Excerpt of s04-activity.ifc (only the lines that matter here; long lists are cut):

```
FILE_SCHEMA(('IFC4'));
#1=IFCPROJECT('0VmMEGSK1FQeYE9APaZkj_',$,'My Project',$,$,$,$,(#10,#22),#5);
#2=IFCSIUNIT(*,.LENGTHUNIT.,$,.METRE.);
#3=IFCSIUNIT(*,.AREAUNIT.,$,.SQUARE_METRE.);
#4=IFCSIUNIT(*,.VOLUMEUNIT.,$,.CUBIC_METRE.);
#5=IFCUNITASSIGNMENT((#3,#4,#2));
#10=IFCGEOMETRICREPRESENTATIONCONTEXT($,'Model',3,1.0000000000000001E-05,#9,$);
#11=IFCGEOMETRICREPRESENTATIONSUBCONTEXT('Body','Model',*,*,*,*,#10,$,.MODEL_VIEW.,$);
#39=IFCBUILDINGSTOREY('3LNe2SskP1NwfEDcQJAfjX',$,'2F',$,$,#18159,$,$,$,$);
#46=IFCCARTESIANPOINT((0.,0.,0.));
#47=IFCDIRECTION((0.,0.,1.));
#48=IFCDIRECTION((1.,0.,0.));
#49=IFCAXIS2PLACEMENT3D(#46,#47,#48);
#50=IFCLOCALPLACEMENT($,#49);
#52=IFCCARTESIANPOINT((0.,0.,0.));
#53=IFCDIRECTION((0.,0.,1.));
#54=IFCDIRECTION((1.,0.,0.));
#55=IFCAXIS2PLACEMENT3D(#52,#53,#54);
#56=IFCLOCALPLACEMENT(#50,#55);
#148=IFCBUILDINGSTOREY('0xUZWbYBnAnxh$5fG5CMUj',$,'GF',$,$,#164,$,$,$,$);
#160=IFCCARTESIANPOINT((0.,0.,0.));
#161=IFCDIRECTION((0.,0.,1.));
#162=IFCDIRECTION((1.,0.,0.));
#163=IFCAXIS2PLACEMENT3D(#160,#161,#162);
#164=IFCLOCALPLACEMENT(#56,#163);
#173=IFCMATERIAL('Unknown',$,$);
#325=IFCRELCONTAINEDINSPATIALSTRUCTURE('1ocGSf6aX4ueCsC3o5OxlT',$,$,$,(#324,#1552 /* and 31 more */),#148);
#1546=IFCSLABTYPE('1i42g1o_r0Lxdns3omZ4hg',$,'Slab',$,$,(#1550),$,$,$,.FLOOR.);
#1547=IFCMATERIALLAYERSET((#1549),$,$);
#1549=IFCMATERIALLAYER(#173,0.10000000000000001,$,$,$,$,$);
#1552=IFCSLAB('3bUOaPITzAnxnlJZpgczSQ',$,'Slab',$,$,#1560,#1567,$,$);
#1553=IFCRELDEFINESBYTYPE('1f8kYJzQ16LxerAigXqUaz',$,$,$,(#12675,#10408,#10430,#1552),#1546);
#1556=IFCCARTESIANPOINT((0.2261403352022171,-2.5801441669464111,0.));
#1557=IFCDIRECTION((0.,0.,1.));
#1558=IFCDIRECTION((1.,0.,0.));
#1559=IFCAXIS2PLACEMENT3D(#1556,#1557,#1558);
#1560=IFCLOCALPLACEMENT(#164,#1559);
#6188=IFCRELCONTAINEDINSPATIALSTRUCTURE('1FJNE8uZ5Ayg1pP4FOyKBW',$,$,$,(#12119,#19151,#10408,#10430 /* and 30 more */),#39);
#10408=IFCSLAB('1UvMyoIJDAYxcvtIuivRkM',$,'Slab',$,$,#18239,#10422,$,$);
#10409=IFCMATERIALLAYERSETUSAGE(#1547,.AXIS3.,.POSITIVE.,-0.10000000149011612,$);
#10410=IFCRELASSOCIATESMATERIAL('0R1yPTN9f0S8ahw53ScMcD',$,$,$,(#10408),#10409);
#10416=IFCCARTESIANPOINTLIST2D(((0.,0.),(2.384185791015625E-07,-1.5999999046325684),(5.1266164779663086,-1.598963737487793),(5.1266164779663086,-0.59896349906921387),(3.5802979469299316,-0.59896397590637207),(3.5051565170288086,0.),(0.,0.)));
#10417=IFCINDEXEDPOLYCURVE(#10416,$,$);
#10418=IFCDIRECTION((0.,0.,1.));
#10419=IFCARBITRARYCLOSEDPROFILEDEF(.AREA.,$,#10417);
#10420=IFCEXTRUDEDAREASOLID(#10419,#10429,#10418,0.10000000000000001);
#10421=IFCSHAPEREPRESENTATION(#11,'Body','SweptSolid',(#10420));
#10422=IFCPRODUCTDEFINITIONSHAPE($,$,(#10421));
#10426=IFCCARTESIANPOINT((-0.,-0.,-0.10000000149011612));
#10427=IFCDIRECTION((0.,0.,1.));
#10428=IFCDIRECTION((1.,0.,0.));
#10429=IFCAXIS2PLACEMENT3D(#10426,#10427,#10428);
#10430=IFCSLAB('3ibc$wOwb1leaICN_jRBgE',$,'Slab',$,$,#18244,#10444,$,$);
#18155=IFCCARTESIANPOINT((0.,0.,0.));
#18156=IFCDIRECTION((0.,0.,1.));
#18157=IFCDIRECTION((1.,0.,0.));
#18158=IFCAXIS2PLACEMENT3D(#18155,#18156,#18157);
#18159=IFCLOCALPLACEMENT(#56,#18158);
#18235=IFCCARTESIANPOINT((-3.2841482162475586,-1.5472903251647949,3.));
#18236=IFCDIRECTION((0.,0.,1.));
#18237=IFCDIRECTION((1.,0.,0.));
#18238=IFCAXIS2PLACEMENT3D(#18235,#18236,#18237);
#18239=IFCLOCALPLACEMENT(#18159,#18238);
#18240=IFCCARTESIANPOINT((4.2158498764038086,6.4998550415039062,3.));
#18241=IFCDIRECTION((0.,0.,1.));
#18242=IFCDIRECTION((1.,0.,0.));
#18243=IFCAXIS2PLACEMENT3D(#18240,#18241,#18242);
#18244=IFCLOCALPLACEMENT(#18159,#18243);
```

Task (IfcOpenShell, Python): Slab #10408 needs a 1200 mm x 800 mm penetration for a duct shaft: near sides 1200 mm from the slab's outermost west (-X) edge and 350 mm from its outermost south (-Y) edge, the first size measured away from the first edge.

```python
import numpy as np
import ifcopenshell
import ifcopenshell.api.feature
import ifcopenshell.api.geometry
import ifcopenshell.api.root
import ifcopenshell.geom
import ifcopenshell.util.placement
import ifcopenshell.util.representation
import ifcopenshell.util.shape
import ifcopenshell.util.unit

model = ifcopenshell.open("s04-activity.ifc")
unit_scale = ifcopenshell.util.unit.calculate_unit_scale(model)
settings = ifcopenshell.geom.settings()


def volume(element):
    """Net volume in cubic metres, openings subtracted."""
    shape = ifcopenshell.geom.create_shape(settings, element)
    return ifcopenshell.util.shape.get_volume(shape.geometry)


slab = model.by_guid("1UvMyoIJDAYxcvtIuivRkM")
before = volume(slab)

# Extent in the slab's own axes, in metres. The edges named are its -X and -Y sides.
slab_shape = ifcopenshell.geom.create_shape(settings, slab)
vertices = ifcopenshell.util.shape.get_vertices(slab_shape.geometry)
x_min, y_min, bottom = vertices.min(axis=0)
top = vertices[:, 2].max()

opening = ifcopenshell.api.root.create_entity(model, ifc_class="IfcOpeningElement", name="Duct shaft opening", predefined_type="OPENING")
context = ifcopenshell.util.representation.get_context(model, "Model", "Body", "MODEL_VIEW")
width, depth = 1.2, 0.8
outline = [(0.0, 0.0), (width, 0.0), (width, depth), (0.0, depth), (0.0, 0.0)]
# Overshoot both faces by 50 mm so the cut is clean.
shape = ifcopenshell.api.geometry.add_slab_representation(
    model, context=context, depth=top - bottom + 0.1, polyline=outline
)
ifcopenshell.api.geometry.assign_representation(model, product=opening, representation=shape)

matrix = ifcopenshell.util.placement.get_local_placement(slab.ObjectPlacement)
matrix[:, 3] = matrix @ np.append(np.array([x_min + 1.2, y_min + 0.35, bottom - 0.05]) / unit_scale, 1.0)
ifcopenshell.api.geometry.edit_object_placement(model, product=opening, matrix=matrix, is_si=False)
ifcopenshell.api.feature.add_feature(model, feature=opening, element=slab)

after = volume(slab)

print(f"slab volume {before:.3f} -> {after:.3f} m3")

model.write("s04-activity_v2.ifc")
```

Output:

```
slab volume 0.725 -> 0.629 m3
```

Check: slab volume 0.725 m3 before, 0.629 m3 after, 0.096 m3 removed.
